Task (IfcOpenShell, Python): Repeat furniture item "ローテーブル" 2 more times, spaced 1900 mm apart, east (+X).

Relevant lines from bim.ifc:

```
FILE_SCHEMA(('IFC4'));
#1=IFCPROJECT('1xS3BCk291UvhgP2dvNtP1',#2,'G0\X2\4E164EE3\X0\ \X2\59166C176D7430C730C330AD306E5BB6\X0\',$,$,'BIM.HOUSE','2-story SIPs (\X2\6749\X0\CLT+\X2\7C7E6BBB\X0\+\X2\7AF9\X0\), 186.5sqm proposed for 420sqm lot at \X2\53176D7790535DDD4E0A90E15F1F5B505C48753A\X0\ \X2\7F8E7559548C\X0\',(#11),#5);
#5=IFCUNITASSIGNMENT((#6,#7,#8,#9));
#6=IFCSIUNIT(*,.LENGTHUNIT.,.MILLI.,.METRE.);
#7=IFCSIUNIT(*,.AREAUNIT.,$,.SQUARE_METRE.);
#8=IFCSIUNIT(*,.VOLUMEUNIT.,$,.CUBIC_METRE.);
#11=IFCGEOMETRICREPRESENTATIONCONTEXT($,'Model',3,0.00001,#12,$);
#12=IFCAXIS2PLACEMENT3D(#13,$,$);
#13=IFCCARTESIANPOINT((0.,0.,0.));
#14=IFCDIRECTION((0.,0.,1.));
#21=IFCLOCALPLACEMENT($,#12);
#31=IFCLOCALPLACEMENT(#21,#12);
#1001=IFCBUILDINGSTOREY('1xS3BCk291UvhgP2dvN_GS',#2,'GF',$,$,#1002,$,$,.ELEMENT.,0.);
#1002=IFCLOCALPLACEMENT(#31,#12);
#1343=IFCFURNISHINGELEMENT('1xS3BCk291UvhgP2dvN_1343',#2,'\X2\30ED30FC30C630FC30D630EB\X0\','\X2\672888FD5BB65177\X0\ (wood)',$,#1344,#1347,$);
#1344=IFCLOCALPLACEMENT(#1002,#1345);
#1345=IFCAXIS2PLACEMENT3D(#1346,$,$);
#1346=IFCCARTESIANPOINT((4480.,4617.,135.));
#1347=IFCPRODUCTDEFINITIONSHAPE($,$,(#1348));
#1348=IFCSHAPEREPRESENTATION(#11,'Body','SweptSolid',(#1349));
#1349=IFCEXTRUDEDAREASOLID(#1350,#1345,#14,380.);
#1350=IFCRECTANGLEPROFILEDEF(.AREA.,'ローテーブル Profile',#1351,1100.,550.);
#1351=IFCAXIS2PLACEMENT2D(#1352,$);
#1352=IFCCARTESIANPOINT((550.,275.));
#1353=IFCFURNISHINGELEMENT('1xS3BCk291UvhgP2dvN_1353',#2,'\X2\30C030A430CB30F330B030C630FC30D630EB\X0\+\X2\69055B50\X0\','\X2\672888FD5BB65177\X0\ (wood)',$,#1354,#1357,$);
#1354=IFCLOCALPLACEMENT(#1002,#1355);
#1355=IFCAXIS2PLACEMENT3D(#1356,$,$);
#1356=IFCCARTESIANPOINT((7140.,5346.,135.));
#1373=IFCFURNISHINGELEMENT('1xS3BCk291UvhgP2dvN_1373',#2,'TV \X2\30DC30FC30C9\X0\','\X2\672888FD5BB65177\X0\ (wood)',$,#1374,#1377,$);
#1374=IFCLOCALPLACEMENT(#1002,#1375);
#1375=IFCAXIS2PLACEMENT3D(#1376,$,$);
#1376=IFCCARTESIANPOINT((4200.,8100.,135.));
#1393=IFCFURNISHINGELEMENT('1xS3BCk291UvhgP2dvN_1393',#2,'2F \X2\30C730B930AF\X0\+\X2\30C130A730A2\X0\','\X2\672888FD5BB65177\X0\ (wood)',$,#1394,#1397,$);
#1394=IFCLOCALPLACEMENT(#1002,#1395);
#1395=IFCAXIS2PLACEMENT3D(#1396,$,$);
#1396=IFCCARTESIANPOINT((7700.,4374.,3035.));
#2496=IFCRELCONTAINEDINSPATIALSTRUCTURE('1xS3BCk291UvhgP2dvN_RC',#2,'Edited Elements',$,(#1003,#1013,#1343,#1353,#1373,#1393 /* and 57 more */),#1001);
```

```python
import numpy as np
import ifcopenshell
import ifcopenshell.api.geometry
import ifcopenshell.api.root
import ifcopenshell.util.element
import ifcopenshell.util.placement
import ifcopenshell.util.unit

model = ifcopenshell.open("bim.ifc")
unit_scale = ifcopenshell.util.unit.calculate_unit_scale(model)


def reuse_history(source, copy):
    """copy_class also copies each property set's owner history, people and application; keep the originals."""
    for rel in copy.IsDefinedBy:
        if rel.is_a("IfcRelDefinesByProperties") and (history := rel.RelatingPropertyDefinition.OwnerHistory):
            rel.RelatingPropertyDefinition.OwnerHistory = source.OwnerHistory
            ifcopenshell.util.element.remove_deep2(model, history)


source = model.by_id(1343)
base = ifcopenshell.util.placement.get_local_placement(source.ObjectPlacement)
step = np.array([1.0, 0.0, 0.0]) * 1.9 / unit_scale

for i in range(1, 3):
    copy = ifcopenshell.api.root.copy_class(model, product=source)
    copy.Representation = ifcopenshell.util.element.copy_deep(
        model, source.Representation, exclude=["IfcGeometricRepresentationContext", "IfcRepresentationMap"]
    )
    reuse_history(source, copy)
    matrix = base.copy()
    matrix[:3, 3] += i * step
    print("added at", matrix[:3, 3].round(3) + 0.0)
    ifcopenshell.api.geometry.edit_object_placement(model, product=copy, matrix=matrix, is_si=False)

model.write("bim_rev.ifc")
```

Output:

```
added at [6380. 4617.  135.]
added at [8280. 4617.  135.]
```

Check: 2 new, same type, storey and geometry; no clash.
